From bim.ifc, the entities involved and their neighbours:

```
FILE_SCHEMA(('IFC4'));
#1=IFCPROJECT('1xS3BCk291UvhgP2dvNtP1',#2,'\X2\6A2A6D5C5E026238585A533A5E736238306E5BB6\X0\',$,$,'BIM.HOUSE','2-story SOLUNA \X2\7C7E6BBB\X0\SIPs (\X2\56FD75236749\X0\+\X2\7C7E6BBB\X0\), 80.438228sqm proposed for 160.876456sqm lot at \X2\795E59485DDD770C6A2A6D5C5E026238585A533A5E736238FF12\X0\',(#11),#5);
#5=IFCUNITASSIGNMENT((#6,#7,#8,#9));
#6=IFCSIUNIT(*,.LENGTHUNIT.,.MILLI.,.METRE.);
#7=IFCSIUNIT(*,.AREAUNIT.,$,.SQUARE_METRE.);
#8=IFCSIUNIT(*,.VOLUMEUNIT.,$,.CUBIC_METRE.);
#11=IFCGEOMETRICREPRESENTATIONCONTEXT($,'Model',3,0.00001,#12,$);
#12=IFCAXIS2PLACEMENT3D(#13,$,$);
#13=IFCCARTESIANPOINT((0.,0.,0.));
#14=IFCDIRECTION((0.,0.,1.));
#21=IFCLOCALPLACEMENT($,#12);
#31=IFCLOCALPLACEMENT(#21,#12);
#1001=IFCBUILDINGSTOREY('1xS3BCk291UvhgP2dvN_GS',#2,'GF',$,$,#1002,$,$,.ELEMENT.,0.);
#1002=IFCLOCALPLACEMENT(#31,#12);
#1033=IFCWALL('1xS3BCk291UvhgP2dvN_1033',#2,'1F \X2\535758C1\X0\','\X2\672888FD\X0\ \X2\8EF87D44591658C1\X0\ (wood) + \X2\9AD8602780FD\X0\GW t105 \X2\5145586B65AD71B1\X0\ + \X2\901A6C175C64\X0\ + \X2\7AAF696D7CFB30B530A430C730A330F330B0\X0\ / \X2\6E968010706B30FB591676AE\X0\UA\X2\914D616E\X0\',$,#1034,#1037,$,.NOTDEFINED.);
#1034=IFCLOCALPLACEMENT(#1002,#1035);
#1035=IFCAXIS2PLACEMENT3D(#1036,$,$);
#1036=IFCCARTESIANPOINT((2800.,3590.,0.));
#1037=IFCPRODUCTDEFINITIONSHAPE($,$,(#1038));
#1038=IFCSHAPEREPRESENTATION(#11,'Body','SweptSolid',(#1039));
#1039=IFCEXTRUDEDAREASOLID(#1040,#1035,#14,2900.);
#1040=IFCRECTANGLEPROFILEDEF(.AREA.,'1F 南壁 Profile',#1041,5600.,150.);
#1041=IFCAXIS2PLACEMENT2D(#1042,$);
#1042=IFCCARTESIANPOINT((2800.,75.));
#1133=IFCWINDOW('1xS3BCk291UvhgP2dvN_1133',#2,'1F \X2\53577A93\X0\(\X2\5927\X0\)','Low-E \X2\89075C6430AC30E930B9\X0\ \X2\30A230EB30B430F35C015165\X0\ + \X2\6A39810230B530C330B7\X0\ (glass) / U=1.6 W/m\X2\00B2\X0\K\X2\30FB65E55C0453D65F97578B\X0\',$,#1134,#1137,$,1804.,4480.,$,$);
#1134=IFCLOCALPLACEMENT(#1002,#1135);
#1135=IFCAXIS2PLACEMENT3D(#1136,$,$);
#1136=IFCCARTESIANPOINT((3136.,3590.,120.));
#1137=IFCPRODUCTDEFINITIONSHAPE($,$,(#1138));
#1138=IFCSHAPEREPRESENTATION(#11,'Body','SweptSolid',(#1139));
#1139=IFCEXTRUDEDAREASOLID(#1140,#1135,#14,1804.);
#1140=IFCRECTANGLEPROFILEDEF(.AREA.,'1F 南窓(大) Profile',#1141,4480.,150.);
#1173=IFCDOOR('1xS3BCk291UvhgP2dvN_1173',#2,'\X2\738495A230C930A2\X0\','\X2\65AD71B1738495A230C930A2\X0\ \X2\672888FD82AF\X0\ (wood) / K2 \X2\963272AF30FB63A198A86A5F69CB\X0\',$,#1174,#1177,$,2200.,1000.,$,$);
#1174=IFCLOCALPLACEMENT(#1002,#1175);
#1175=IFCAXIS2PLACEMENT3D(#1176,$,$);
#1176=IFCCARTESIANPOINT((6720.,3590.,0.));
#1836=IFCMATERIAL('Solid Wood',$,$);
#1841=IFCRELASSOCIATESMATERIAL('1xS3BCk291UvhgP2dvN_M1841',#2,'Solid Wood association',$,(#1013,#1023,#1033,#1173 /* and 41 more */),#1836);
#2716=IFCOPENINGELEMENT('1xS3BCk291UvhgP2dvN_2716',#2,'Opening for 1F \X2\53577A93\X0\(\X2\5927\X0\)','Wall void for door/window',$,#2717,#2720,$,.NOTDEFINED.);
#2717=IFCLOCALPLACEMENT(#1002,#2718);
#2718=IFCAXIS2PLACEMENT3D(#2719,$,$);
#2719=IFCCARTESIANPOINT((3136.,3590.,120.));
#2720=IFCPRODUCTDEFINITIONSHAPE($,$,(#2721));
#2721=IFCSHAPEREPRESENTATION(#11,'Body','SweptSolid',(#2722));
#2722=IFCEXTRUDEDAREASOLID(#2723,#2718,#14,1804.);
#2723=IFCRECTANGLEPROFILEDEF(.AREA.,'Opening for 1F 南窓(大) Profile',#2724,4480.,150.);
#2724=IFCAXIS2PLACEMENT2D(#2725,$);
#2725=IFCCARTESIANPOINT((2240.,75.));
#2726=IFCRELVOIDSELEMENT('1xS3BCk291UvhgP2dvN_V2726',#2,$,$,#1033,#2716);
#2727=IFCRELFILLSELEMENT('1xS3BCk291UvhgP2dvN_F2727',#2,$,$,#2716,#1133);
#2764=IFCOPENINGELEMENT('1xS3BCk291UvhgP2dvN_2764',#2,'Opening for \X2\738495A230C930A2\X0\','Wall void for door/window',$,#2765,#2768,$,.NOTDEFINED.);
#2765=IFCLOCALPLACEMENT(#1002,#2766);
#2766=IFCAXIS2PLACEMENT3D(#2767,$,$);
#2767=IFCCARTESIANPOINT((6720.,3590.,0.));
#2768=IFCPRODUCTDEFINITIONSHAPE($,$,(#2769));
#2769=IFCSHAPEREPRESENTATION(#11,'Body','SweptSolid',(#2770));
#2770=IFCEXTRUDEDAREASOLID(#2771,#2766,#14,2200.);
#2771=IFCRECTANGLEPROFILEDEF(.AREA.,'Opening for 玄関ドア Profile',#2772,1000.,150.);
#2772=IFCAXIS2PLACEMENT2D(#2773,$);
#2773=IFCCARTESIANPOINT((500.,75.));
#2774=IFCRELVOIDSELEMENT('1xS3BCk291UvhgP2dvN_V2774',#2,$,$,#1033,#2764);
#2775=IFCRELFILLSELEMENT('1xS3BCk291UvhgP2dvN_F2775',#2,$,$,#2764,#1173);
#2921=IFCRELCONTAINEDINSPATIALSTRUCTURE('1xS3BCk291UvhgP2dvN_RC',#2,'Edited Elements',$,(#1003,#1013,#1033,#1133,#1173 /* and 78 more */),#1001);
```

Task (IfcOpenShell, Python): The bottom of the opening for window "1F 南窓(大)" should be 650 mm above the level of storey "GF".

```python
import numpy as np
import ifcopenshell
import ifcopenshell.api.geometry
import ifcopenshell.geom
import ifcopenshell.util.element
import ifcopenshell.util.placement
import ifcopenshell.util.shape
import ifcopenshell.util.unit

model = ifcopenshell.open("bim.ifc")
unit_scale = ifcopenshell.util.unit.calculate_unit_scale(model)

window = model.by_guid("1xS3BCk291UvhgP2dvN_1133")
opening = window.FillsVoids[0].RelatingOpeningElement
storey = ifcopenshell.util.element.get_container(window, ifc_class="IfcBuildingStorey")
level = ifcopenshell.util.placement.get_local_placement(storey.ObjectPlacement)[2, 3]

# The opening's origin need not be at the sill, so measure its lowest point.
shape = ifcopenshell.geom.create_shape(ifcopenshell.geom.settings(), opening)
bottom = ifcopenshell.util.shape.get_shape_bottom_elevation(shape, shape.geometry) / unit_scale
dz = level + 0.65 / unit_scale - bottom

shift = np.array([0.0, 0.0, dz])
# The window is not placed relative to its opening, so move both.
for product in (opening, window):
    matrix = ifcopenshell.util.placement.get_local_placement(product.ObjectPlacement)
    matrix[:3, 3] += shift
    ifcopenshell.api.geometry.edit_object_placement(model, product=product, matrix=matrix, is_si=False)

print(f"moved by {dz * unit_scale:+.3f} m")

model.write("bim-out.ifc")
```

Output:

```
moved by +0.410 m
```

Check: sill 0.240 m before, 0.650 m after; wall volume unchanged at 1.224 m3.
